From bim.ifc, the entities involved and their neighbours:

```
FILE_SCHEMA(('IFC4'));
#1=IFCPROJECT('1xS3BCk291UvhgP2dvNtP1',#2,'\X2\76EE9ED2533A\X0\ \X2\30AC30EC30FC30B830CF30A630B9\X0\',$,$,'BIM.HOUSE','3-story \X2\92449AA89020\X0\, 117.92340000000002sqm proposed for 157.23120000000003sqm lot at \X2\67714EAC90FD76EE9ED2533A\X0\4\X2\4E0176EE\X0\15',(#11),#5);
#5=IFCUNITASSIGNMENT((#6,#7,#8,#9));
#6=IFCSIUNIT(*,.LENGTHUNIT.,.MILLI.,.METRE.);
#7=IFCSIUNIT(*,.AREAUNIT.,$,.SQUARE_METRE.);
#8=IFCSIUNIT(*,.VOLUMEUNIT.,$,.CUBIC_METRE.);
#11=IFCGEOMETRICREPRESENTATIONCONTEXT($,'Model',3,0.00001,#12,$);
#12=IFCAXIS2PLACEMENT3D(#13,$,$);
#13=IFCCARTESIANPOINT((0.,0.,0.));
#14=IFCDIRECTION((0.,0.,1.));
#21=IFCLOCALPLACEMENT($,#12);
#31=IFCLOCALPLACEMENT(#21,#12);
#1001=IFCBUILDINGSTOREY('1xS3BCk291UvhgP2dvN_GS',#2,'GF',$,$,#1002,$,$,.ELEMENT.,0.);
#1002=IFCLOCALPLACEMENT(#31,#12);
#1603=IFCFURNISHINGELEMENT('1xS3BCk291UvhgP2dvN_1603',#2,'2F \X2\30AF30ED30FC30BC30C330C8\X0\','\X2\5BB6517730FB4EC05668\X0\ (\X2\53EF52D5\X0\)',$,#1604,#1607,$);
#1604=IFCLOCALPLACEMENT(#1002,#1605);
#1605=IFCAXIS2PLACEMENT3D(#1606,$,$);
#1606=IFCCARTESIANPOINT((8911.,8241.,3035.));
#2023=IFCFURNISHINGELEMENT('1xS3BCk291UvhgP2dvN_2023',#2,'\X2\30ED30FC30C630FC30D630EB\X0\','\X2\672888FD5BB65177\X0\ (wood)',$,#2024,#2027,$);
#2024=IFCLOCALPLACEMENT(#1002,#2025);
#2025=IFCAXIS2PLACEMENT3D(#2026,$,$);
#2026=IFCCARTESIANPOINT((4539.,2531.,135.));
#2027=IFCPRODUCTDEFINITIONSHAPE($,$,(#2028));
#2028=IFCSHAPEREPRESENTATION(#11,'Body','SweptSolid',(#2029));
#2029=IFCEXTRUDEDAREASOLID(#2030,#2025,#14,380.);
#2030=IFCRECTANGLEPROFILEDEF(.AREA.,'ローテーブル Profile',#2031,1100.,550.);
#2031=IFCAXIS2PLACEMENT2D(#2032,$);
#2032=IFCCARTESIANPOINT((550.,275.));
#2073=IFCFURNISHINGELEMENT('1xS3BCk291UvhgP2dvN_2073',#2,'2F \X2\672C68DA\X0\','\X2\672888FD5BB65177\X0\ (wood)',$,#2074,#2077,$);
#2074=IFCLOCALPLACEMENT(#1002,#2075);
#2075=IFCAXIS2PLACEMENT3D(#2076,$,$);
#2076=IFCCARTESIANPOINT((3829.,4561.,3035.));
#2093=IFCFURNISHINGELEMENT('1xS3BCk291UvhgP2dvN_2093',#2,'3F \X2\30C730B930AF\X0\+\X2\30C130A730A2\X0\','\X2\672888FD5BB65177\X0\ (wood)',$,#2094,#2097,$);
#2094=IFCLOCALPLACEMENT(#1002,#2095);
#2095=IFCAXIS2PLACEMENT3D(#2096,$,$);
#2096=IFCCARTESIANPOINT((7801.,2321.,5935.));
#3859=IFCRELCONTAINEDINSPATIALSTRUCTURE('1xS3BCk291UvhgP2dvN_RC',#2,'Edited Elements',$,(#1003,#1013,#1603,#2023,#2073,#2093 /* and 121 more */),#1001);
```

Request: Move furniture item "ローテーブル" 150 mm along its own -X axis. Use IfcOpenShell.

```python
import ifcopenshell
import ifcopenshell.api.geometry
import ifcopenshell.util.placement
import ifcopenshell.util.unit

model = ifcopenshell.open("bim.ifc")
unit_scale = ifcopenshell.util.unit.calculate_unit_scale(model)

item = model.by_guid("1xS3BCk291UvhgP2dvN_2023")
matrix = ifcopenshell.util.placement.get_local_placement(item.ObjectPlacement)
matrix[:3, 3] -= matrix[:3, 0] * 0.15 / unit_scale
ifcopenshell.api.geometry.edit_object_placement(model, product=item, matrix=matrix, is_si=False)

print(ifcopenshell.util.placement.get_local_placement(item.ObjectPlacement).round(3) + 0.0)

model.write("bim_updated.ifc")
```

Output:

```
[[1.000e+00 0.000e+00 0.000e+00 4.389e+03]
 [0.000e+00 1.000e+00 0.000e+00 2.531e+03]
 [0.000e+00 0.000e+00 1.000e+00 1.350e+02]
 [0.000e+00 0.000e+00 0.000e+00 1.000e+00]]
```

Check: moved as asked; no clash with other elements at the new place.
